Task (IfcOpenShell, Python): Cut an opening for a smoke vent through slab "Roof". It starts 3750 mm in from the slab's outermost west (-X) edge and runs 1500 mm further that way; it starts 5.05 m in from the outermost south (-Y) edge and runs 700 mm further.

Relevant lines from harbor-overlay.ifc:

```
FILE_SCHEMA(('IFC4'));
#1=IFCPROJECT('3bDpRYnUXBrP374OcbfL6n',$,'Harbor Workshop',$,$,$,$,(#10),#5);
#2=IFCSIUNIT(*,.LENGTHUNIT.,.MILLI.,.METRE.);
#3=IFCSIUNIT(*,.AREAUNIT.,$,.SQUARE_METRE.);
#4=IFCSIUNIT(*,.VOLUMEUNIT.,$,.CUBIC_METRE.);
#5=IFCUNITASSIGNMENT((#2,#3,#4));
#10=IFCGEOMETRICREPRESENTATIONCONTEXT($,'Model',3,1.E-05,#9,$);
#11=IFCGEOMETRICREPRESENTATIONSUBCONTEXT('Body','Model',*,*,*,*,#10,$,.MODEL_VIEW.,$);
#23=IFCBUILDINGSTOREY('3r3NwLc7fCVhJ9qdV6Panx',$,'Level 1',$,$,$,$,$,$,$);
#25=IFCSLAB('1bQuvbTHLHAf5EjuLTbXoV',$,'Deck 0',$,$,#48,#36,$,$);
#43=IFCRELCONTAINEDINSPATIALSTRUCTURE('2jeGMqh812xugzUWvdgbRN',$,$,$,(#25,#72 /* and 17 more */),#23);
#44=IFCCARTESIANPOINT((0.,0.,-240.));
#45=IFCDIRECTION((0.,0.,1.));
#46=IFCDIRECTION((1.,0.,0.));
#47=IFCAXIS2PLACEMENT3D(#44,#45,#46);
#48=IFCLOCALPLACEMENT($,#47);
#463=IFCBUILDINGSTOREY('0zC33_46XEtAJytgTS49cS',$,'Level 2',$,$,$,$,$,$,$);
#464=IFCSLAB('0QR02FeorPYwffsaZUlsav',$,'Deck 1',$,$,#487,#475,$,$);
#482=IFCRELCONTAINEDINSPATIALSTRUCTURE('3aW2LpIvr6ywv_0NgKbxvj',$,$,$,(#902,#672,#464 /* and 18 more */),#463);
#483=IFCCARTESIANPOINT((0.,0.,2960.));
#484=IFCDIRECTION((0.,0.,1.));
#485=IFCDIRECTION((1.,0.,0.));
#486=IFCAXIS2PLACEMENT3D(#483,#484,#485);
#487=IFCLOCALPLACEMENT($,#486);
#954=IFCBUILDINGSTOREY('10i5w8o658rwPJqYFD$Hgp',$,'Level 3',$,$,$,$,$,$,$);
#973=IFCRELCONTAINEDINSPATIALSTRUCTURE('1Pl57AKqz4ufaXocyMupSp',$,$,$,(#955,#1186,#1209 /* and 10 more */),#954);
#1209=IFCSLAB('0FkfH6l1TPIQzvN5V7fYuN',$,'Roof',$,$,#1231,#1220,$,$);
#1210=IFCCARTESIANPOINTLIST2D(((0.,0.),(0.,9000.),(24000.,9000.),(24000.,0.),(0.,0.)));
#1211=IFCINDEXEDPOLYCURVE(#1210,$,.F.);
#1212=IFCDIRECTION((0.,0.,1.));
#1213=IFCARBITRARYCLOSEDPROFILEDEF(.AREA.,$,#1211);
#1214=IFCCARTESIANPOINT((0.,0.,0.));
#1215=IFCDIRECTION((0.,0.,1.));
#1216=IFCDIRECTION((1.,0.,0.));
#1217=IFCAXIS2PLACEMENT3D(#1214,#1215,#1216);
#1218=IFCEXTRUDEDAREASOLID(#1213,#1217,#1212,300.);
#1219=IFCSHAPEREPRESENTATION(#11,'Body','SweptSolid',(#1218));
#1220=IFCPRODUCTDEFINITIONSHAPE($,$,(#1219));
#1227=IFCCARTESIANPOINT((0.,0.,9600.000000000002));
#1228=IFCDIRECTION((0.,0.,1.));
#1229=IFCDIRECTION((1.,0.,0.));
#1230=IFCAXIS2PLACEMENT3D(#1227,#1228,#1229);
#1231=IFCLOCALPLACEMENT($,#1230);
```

```python
import numpy as np
import ifcopenshell
import ifcopenshell.api.feature
import ifcopenshell.api.geometry
import ifcopenshell.api.root
import ifcopenshell.geom
import ifcopenshell.util.placement
import ifcopenshell.util.representation
import ifcopenshell.util.shape
import ifcopenshell.util.unit

model = ifcopenshell.open("harbor-overlay.ifc")
unit_scale = ifcopenshell.util.unit.calculate_unit_scale(model)
settings = ifcopenshell.geom.settings()


def volume(element):
    """Net volume in cubic metres, openings subtracted."""
    shape = ifcopenshell.geom.create_shape(settings, element)
    return ifcopenshell.util.shape.get_volume(shape.geometry)


slab = model.by_id(1209)
before = volume(slab)

# Extent in the slab's own axes, in metres. The edges named are its -X and -Y sides.
slab_shape = ifcopenshell.geom.create_shape(settings, slab)
vertices = ifcopenshell.util.shape.get_vertices(slab_shape.geometry)
x_min, y_min, bottom = vertices.min(axis=0)
top = vertices[:, 2].max()

opening = ifcopenshell.api.root.create_entity(model, ifc_class="IfcOpeningElement", name="Smoke vent opening", predefined_type="OPENING")
context = ifcopenshell.util.representation.get_context(model, "Model", "Body", "MODEL_VIEW")
width, depth = 1.5, 0.7
outline = [(0.0, 0.0), (width, 0.0), (width, depth), (0.0, depth), (0.0, 0.0)]
# Overshoot both faces by 50 mm so the cut is clean.
shape = ifcopenshell.api.geometry.add_slab_representation(
    model, context=context, depth=top - bottom + 0.1, polyline=outline
)
ifcopenshell.api.geometry.assign_representation(model, product=opening, representation=shape)

matrix = ifcopenshell.util.placement.get_local_placement(slab.ObjectPlacement)
matrix[:, 3] = matrix @ np.append(np.array([x_min + 3.75, y_min + 5.05, bottom - 0.05]) / unit_scale, 1.0)
ifcopenshell.api.geometry.edit_object_placement(model, product=opening, matrix=matrix, is_si=False)
ifcopenshell.api.feature.add_feature(model, feature=opening, element=slab)

after = volume(slab)

print(f"slab volume {before:.3f} -> {after:.3f} m3")

model.write("harbor-overlay_v2.ifc")
```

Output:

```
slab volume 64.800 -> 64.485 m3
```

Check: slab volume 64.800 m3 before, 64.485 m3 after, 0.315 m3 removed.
